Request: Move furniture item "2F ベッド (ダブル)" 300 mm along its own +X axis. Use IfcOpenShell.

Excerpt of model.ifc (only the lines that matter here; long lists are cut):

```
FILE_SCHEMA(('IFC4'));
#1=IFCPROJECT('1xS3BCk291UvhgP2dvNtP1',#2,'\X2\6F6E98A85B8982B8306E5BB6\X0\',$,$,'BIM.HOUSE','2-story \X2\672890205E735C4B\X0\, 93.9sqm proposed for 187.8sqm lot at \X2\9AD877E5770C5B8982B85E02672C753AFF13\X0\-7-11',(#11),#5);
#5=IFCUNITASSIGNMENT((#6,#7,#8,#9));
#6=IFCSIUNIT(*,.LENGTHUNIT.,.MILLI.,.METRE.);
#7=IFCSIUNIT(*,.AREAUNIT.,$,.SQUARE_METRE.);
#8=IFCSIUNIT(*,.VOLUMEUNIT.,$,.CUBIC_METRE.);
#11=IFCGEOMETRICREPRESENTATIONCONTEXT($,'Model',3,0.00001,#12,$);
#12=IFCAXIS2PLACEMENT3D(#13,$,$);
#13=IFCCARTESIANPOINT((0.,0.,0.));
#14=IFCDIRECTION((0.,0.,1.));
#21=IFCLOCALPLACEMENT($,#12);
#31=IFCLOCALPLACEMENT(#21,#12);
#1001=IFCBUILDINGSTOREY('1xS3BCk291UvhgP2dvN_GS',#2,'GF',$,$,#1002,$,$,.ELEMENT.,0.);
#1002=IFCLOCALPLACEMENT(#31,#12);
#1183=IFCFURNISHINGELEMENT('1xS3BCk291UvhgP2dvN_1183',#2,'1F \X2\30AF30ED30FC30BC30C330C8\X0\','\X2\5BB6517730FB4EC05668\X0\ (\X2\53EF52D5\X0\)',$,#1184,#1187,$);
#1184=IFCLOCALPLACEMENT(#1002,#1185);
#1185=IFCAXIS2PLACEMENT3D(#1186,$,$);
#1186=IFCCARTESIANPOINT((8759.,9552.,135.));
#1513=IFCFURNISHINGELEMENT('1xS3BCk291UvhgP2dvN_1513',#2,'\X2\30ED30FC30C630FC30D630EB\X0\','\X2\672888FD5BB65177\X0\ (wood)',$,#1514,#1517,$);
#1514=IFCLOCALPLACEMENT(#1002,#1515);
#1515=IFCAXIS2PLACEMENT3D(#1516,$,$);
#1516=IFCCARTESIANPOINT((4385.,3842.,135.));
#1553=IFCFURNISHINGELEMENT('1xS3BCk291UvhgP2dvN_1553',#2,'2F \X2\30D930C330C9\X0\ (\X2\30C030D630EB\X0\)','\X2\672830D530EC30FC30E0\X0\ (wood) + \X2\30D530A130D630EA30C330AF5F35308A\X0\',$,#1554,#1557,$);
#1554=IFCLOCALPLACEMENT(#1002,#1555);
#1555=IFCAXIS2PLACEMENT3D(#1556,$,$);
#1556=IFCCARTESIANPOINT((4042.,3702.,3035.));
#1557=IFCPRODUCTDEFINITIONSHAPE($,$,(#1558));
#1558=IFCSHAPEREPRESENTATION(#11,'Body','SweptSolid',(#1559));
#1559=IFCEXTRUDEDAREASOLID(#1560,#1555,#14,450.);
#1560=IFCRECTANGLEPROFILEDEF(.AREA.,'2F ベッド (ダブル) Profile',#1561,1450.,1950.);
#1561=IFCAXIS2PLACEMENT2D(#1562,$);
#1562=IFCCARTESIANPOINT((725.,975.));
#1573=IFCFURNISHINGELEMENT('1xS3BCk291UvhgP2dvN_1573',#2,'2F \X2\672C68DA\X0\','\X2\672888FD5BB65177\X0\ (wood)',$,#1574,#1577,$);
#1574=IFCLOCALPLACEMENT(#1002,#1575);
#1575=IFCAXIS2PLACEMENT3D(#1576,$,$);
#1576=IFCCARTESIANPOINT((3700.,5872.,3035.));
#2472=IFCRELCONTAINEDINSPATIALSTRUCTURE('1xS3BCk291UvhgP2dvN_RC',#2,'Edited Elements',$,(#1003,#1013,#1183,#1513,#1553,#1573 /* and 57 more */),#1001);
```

```python
import ifcopenshell
import ifcopenshell.api.geometry
import ifcopenshell.util.placement

model = ifcopenshell.open("model.ifc")

item = model.by_guid("1xS3BCk291UvhgP2dvN_1553")
matrix = ifcopenshell.util.placement.get_local_placement(item.ObjectPlacement)
matrix[:3, 3] += matrix[:3, 0] * 300.0
ifcopenshell.api.geometry.edit_object_placement(model, product=item, matrix=matrix, is_si=False)

print(ifcopenshell.util.placement.get_local_placement(item.ObjectPlacement).round(3) + 0.0)

model.write("model-out.ifc")
```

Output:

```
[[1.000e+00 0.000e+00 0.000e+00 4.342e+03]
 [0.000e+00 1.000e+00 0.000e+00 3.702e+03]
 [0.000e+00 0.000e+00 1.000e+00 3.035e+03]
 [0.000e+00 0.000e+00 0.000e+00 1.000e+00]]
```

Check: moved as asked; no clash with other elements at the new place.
